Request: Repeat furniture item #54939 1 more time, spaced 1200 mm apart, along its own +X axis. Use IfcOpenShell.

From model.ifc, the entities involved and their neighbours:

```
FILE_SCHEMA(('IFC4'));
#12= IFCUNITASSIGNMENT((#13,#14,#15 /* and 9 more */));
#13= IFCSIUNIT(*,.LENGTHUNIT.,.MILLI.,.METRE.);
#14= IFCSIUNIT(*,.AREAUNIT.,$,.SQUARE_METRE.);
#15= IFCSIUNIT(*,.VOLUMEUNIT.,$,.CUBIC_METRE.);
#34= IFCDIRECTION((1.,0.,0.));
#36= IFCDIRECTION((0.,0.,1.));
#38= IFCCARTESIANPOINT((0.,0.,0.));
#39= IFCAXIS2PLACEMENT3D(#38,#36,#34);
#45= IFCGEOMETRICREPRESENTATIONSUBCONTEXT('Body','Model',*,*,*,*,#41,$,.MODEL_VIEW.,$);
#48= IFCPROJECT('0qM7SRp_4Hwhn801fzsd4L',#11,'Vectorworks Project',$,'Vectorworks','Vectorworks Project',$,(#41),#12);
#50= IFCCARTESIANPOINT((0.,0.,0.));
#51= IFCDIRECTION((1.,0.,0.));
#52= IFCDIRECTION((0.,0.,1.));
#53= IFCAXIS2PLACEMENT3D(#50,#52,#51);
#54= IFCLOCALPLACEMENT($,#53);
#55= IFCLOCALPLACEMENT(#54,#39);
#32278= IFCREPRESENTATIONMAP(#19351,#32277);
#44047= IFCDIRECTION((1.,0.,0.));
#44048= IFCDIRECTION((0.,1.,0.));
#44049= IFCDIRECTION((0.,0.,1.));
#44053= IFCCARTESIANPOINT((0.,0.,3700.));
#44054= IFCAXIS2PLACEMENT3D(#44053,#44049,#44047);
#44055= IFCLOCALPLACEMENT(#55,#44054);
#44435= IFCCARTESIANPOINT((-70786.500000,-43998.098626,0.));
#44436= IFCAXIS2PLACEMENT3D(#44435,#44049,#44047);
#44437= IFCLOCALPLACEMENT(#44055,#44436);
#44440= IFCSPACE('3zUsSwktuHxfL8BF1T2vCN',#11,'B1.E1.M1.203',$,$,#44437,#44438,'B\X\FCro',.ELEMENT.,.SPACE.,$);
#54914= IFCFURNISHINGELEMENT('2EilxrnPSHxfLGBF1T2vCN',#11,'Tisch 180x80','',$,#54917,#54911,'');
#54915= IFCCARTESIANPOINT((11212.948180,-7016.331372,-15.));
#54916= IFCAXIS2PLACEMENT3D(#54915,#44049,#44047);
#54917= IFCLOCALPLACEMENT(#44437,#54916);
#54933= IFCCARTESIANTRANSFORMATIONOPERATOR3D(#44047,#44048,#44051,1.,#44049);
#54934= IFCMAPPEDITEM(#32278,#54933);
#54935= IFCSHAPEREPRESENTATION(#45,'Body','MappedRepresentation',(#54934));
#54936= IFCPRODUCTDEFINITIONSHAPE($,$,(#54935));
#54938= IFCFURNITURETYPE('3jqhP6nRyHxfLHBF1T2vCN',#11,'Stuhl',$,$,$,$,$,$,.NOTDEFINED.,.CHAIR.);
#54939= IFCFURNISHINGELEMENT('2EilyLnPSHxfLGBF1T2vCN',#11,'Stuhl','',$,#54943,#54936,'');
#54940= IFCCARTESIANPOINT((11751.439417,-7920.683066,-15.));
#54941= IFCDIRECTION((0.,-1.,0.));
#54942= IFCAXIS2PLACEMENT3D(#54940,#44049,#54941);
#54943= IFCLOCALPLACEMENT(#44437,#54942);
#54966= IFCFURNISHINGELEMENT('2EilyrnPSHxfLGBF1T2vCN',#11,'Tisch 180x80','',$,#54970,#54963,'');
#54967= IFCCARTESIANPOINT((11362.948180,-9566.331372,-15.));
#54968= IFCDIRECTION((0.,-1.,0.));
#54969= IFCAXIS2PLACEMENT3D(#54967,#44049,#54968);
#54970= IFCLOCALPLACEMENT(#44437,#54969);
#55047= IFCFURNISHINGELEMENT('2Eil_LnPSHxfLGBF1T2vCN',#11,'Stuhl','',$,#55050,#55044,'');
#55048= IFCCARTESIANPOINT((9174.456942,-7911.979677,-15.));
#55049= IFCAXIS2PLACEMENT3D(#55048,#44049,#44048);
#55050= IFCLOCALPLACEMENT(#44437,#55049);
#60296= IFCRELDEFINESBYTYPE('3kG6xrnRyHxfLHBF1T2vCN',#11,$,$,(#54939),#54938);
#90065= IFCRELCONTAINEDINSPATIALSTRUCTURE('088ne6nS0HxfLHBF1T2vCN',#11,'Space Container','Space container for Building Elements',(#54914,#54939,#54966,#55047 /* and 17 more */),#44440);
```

```python
import ifcopenshell
import ifcopenshell.api.geometry
import ifcopenshell.api.root
import ifcopenshell.util.element
import ifcopenshell.util.placement

model = ifcopenshell.open("model.ifc")

source = model.by_id(54939)
base = ifcopenshell.util.placement.get_local_placement(source.ObjectPlacement)
step = base[:3, 0] * 1200.0

for i in range(1, 2):
    copy = ifcopenshell.api.root.copy_class(model, product=source)
    copy.Representation = ifcopenshell.util.element.copy_deep(
        model, source.Representation, exclude=["IfcGeometricRepresentationContext", "IfcRepresentationMap"]
    )
    matrix = base.copy()
    matrix[:3, 3] += i * step
    print("added at", matrix[:3, 3].round(3) + 0.0)
    ifcopenshell.api.geometry.edit_object_placement(model, product=copy, matrix=matrix, is_si=False)

model.write("model_v2.ifc")
```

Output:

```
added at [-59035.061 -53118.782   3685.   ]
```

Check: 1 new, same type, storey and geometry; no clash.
